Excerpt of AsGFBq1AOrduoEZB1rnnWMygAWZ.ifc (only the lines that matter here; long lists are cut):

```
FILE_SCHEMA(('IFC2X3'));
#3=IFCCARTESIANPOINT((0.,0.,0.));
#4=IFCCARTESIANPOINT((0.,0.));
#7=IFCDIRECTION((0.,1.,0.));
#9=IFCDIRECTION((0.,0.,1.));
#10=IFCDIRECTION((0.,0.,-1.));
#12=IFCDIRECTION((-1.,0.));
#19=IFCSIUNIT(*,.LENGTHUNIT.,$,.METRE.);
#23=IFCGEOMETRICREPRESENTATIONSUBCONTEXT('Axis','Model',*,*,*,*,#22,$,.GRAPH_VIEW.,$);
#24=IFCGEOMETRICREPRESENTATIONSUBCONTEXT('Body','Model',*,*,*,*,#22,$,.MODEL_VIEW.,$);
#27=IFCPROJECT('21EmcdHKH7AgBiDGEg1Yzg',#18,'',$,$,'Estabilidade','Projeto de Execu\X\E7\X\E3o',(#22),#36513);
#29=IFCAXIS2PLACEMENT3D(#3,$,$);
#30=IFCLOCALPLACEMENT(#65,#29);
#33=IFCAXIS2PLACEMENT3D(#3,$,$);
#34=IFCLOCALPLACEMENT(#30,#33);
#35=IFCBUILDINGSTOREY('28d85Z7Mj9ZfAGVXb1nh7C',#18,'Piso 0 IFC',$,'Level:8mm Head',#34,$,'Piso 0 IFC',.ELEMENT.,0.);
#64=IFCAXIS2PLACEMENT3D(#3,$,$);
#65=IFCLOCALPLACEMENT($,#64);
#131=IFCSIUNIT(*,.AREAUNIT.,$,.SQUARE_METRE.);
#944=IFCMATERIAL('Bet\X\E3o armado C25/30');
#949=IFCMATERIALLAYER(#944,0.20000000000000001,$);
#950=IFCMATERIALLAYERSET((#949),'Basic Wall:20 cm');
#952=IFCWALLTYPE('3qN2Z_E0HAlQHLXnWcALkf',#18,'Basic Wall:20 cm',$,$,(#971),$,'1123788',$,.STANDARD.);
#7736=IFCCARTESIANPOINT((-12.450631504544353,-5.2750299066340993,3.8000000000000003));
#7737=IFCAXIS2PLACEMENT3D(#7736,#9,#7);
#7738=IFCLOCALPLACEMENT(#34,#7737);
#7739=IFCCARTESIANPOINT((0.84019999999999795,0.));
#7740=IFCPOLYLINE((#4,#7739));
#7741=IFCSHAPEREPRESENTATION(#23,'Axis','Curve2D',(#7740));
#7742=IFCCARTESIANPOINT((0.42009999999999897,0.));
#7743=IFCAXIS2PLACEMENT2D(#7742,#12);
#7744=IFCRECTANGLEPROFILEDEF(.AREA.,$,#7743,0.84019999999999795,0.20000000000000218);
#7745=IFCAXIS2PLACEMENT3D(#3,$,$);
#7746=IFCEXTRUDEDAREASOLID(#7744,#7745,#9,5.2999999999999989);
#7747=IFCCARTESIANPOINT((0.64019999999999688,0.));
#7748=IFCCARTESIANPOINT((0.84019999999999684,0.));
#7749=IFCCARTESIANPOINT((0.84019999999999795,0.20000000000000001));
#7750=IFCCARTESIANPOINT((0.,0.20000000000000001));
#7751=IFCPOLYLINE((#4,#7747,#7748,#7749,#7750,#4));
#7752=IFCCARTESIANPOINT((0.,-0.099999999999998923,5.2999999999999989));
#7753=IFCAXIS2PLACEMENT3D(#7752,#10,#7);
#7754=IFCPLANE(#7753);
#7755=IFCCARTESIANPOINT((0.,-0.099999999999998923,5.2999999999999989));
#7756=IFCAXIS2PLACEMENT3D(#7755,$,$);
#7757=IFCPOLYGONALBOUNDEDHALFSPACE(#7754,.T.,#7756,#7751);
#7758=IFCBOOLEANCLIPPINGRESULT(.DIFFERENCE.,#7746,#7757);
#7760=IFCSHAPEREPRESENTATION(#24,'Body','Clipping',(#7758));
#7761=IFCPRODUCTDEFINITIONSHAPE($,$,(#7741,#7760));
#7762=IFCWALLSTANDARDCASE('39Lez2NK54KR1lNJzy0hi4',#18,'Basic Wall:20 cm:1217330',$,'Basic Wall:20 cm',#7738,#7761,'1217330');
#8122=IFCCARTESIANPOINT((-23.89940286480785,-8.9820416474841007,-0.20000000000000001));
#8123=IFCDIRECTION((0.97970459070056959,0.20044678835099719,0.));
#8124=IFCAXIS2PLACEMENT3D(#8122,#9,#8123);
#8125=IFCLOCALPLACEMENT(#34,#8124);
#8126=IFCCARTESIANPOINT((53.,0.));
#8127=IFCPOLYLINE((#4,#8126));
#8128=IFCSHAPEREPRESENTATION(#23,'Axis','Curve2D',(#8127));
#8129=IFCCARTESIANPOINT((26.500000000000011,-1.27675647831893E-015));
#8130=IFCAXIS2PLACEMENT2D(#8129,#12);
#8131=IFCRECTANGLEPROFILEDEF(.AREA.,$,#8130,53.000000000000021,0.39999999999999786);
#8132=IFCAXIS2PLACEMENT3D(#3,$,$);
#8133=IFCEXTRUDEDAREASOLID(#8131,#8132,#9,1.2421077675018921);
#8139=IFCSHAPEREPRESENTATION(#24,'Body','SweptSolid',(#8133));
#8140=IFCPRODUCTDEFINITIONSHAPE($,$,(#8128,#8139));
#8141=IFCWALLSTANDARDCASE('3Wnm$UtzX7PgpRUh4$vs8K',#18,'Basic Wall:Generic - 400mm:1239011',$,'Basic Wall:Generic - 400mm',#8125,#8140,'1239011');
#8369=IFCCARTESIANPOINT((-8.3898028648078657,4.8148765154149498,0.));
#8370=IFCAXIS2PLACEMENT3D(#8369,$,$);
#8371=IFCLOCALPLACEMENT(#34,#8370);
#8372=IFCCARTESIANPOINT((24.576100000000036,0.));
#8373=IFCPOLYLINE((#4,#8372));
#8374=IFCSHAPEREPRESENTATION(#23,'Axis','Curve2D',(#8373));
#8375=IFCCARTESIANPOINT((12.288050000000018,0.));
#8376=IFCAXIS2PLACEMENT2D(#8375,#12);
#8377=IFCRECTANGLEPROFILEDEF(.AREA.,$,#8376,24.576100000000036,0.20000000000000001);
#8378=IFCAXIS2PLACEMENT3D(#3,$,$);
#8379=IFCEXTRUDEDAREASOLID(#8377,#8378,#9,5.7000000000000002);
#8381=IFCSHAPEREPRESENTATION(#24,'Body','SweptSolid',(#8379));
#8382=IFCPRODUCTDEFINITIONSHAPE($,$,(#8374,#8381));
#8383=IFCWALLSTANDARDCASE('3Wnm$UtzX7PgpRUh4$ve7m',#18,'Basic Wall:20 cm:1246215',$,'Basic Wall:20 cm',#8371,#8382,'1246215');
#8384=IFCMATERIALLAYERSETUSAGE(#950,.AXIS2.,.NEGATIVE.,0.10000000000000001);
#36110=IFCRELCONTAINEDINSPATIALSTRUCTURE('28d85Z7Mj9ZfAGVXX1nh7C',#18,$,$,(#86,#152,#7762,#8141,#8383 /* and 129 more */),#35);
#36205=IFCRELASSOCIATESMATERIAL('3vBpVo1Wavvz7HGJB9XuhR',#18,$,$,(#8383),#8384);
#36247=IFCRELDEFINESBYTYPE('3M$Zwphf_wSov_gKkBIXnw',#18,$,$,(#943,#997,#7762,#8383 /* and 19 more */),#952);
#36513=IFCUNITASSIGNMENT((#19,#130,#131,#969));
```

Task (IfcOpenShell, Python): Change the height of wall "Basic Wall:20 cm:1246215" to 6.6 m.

```python
import ifcopenshell
import ifcopenshell.geom
import ifcopenshell.util.representation
import ifcopenshell.util.shape
import ifcopenshell.util.unit

model = ifcopenshell.open("AsGFBq1AOrduoEZB1rnnWMygAWZ.ifc")
unit_scale = ifcopenshell.util.unit.calculate_unit_scale(model)
settings = ifcopenshell.geom.settings()


def volume(element):
    """Net volume in cubic metres, openings subtracted."""
    shape = ifcopenshell.geom.create_shape(settings, element)
    return ifcopenshell.util.shape.get_volume(shape.geometry)


wall = model.by_guid("3Wnm$UtzX7PgpRUh4$ve7m")
before = volume(wall)

body = ifcopenshell.util.representation.get_representation(wall, "Model", "Body")
solid = body.Items[0]
old_height = solid.Depth
solid.Depth = 6.6 / unit_scale
after = volume(wall)

print(f"height {old_height:g} -> {solid.Depth:g}, volume {before:.3f} -> {after:.3f} m3")

model.write("AsGFBq1AOrduoEZB1rnnWMygAWZ_rev.ifc")
```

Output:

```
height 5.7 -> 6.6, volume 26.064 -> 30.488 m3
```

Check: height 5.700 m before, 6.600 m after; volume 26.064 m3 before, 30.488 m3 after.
